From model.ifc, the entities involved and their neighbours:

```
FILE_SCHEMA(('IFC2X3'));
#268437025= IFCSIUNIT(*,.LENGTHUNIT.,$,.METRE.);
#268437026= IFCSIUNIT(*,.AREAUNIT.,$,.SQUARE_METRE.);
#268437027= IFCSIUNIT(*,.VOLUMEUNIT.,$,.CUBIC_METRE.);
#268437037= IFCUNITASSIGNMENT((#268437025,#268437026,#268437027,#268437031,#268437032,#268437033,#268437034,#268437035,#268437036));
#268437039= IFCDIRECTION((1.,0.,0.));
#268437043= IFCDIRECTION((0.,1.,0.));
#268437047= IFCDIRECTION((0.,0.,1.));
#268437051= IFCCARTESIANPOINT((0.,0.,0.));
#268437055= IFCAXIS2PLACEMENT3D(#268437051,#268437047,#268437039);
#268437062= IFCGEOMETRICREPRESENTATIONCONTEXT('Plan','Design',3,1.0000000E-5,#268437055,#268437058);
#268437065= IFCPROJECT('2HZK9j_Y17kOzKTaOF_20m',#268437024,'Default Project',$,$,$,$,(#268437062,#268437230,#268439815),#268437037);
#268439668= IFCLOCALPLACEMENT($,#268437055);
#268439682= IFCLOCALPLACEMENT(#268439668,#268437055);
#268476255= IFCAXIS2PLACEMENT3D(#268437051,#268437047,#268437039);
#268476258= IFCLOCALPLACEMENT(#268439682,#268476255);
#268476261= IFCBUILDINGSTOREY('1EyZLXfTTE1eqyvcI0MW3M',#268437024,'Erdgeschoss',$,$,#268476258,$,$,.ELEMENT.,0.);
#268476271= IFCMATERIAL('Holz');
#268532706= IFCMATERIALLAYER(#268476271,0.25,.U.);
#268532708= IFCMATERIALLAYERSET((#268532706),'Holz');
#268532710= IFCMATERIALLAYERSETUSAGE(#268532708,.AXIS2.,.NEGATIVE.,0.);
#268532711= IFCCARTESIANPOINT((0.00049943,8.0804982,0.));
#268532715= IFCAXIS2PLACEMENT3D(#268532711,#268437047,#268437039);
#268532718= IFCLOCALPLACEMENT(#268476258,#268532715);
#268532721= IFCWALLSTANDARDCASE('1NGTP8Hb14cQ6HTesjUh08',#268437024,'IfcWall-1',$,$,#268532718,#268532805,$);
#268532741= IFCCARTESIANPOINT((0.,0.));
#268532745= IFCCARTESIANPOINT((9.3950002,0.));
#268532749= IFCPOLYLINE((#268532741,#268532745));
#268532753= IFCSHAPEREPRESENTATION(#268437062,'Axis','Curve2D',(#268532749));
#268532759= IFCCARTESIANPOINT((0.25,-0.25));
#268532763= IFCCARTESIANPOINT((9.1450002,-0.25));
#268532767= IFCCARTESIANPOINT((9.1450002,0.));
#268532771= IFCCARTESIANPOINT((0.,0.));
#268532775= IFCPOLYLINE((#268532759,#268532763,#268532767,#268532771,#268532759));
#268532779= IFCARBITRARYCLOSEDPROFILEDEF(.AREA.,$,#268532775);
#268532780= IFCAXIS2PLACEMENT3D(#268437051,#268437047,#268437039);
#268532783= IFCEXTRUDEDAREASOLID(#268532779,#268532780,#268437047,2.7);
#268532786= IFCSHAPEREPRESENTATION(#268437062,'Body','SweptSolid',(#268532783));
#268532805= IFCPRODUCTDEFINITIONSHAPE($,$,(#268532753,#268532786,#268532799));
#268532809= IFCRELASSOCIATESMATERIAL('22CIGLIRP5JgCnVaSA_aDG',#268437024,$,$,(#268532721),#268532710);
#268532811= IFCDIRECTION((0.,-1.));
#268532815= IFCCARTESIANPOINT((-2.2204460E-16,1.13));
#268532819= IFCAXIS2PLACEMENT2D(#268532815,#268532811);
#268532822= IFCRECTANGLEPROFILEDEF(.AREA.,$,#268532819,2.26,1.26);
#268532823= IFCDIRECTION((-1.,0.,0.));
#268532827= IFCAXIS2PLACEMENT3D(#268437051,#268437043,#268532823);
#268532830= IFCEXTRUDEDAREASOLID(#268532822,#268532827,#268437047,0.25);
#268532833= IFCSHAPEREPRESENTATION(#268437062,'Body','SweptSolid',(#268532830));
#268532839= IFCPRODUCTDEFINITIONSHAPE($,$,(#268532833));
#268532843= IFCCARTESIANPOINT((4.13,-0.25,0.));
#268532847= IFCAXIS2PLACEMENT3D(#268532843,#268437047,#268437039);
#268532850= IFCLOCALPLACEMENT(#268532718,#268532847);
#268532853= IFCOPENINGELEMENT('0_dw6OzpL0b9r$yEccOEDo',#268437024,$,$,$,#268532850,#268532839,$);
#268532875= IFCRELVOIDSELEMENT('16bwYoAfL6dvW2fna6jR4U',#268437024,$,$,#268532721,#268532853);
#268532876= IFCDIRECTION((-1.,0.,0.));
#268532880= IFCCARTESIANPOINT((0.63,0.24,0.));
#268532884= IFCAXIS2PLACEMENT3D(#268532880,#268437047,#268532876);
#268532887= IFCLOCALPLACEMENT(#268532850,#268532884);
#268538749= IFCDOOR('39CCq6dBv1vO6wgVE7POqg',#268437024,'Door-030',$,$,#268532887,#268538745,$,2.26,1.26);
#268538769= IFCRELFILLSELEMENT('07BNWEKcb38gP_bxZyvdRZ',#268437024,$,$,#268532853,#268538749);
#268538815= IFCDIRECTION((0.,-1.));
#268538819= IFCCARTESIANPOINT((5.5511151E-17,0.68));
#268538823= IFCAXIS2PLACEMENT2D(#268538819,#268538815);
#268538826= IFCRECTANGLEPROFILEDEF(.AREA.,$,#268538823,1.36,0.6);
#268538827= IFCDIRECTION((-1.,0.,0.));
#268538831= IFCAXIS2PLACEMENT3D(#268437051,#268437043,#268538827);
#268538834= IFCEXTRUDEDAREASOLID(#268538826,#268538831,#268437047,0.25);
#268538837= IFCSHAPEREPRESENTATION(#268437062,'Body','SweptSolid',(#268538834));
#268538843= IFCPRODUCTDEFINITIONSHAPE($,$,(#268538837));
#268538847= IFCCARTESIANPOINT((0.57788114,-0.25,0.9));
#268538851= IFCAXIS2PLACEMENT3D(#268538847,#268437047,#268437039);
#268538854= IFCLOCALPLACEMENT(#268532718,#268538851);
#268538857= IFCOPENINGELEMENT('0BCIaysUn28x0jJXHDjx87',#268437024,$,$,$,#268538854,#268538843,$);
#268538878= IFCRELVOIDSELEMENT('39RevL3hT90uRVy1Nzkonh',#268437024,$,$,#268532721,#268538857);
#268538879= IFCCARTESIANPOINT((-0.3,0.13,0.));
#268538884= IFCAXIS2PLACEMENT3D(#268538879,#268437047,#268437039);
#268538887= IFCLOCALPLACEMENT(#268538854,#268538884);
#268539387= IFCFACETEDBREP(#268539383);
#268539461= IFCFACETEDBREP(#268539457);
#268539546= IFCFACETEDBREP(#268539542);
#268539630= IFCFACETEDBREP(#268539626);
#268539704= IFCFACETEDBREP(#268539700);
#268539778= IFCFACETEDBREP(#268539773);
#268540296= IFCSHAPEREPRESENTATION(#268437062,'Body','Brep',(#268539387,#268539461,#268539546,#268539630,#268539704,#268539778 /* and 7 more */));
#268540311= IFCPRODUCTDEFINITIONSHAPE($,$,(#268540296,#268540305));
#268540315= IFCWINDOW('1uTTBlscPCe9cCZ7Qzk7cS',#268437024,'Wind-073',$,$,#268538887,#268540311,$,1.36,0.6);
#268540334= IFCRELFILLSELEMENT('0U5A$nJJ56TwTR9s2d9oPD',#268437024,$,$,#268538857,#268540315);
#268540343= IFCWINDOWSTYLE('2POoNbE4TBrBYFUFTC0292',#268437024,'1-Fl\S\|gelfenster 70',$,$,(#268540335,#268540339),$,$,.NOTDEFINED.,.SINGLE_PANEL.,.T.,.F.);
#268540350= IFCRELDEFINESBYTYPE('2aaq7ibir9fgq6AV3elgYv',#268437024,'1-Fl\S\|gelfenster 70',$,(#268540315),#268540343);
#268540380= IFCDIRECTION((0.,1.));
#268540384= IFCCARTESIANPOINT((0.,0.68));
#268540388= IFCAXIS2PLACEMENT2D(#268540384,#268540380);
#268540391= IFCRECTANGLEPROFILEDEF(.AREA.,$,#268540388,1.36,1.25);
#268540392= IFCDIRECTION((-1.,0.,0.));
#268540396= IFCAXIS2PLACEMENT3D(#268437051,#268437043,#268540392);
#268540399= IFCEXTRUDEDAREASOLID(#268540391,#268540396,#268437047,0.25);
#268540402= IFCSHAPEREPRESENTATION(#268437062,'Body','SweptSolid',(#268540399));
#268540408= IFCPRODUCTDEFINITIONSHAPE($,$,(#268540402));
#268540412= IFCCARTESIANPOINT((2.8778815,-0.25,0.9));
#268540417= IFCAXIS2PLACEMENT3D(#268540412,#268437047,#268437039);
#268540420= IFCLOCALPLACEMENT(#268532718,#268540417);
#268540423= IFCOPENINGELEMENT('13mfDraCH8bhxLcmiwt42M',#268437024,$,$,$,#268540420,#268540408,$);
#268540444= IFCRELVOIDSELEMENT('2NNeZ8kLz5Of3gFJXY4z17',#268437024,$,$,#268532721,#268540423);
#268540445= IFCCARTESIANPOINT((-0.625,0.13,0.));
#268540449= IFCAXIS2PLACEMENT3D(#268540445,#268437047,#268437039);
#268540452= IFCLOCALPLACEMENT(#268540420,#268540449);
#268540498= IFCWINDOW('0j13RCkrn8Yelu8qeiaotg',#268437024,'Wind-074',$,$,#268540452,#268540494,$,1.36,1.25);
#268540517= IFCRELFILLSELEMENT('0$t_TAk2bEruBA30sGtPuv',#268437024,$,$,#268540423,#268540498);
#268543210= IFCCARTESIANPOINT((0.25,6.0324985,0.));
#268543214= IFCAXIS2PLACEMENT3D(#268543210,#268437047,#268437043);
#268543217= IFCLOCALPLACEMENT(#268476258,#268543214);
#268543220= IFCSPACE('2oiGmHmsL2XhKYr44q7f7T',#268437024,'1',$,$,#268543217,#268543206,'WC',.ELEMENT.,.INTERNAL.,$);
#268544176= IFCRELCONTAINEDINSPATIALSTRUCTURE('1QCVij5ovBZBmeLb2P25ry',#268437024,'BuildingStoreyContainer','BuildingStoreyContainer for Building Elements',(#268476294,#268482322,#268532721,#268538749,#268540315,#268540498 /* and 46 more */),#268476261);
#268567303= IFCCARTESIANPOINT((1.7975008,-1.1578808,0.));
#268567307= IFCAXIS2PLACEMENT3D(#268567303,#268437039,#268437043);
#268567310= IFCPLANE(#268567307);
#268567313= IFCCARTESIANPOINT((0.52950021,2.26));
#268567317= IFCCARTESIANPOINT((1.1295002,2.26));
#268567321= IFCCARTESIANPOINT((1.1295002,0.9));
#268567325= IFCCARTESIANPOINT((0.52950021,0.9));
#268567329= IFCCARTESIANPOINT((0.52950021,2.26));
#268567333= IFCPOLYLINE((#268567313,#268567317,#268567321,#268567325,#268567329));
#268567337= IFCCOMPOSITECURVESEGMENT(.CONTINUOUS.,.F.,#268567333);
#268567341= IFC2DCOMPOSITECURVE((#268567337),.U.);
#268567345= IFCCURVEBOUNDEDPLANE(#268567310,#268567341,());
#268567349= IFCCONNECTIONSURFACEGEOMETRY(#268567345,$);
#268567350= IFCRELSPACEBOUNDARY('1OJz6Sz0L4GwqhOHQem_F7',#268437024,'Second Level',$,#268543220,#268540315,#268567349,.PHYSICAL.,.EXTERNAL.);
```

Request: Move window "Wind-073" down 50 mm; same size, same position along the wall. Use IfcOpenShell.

```python
import numpy as np
import ifcopenshell
import ifcopenshell.api.geometry
import ifcopenshell.util.placement
import ifcopenshell.util.unit

model = ifcopenshell.open("model.ifc")
unit_scale = ifcopenshell.util.unit.calculate_unit_scale(model)

window = model.by_guid("1uTTBlscPCe9cCZ7Qzk7cS")
opening = window.FillsVoids[0].RelatingOpeningElement
dz = -0.05 / unit_scale

shift = np.array([0.0, 0.0, dz])
# The window is placed relative to its opening, so it follows when the opening moves.
matrix = ifcopenshell.util.placement.get_local_placement(opening.ObjectPlacement)
matrix[:3, 3] += shift
ifcopenshell.api.geometry.edit_object_placement(
    model, product=opening, matrix=matrix, is_si=False, should_transform_children=True
)

# Space boundary surfaces are stored in each space's coordinates; move them too.
for rel in window.ProvidesBoundaries:
    if not rel.ConnectionGeometry:
        continue
    surface = rel.ConnectionGeometry.SurfaceOnRelatingElement.BasisSurface
    space_matrix = ifcopenshell.util.placement.get_local_placement(rel.RelatingSpace.ObjectPlacement)
    point = np.array(surface.Position.Location.Coordinates) + space_matrix[:3, :3].T @ shift
    surface.Position = model.createIfcAxis2Placement3D(
        model.createIfcCartesianPoint(point.tolist()), surface.Position.Axis, surface.Position.RefDirection
    )

print(f"moved by {dz * unit_scale:+.3f} m")

model.write("model_updated.ifc")
```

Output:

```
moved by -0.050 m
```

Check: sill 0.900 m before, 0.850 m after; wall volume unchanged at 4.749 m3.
